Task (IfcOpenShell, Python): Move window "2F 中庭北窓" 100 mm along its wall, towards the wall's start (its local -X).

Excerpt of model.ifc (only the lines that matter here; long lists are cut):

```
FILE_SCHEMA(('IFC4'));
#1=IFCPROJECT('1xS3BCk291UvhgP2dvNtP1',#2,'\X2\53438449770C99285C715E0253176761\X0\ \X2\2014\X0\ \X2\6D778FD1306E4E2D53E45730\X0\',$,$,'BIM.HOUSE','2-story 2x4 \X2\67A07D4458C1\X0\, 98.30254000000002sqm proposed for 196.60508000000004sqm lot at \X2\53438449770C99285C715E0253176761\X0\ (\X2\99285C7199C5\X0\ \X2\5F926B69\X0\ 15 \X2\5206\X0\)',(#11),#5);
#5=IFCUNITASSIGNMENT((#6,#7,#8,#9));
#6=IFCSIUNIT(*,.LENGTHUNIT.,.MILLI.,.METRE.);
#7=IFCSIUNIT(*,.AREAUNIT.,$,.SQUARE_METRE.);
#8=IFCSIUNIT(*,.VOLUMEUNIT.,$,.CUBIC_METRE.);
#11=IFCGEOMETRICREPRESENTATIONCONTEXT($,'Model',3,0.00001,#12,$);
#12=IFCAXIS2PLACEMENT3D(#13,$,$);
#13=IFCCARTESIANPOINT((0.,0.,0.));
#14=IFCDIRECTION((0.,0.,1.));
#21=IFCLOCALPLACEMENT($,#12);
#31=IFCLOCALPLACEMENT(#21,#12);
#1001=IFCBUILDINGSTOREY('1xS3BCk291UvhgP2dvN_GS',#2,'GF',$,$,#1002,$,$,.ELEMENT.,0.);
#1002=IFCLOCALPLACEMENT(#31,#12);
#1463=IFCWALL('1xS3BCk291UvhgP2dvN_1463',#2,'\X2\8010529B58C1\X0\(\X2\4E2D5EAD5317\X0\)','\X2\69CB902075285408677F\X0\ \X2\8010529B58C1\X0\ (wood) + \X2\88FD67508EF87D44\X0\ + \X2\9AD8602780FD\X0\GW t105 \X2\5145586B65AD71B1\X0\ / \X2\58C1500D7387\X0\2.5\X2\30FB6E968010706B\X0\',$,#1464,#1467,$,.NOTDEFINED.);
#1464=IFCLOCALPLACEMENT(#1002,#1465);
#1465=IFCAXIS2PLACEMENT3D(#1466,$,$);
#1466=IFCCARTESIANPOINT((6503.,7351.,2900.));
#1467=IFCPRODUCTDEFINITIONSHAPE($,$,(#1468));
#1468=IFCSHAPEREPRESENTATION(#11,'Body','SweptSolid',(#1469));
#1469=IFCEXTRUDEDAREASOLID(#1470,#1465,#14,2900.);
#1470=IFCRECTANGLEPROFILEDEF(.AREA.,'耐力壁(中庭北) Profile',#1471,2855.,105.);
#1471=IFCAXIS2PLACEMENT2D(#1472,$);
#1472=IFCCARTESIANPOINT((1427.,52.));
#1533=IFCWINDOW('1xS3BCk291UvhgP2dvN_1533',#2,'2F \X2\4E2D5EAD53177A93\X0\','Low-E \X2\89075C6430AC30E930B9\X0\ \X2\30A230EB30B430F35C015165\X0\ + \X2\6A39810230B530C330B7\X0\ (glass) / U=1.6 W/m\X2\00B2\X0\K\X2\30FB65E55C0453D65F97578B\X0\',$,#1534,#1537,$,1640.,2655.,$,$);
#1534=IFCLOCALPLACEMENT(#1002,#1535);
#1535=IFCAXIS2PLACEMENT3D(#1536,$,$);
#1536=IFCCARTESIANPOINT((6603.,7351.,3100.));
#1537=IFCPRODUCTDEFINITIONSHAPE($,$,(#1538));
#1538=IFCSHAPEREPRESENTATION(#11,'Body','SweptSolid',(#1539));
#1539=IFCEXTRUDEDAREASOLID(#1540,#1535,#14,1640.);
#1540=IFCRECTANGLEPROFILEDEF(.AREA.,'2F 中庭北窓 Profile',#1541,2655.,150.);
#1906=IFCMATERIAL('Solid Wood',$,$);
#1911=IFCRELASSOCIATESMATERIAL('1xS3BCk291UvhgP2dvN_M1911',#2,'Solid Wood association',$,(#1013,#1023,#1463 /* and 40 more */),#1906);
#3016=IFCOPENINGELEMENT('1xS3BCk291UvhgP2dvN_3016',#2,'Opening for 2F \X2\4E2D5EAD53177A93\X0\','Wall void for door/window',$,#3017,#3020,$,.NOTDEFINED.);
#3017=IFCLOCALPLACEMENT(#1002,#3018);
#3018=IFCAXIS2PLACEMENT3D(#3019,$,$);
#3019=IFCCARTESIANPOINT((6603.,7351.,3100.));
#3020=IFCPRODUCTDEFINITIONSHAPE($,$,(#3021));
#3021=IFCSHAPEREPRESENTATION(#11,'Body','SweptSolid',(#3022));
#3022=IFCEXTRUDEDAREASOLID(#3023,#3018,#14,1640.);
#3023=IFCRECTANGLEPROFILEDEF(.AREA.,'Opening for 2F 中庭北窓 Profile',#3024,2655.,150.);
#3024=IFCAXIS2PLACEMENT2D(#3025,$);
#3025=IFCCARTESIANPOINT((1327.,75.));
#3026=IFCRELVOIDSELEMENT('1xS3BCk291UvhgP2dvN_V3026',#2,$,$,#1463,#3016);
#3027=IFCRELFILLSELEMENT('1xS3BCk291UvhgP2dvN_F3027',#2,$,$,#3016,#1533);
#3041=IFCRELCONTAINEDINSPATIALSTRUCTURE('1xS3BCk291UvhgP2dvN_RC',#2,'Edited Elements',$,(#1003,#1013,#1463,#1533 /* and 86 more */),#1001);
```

```python
import ifcopenshell
import ifcopenshell.api.geometry
import ifcopenshell.util.placement
import ifcopenshell.util.unit

model = ifcopenshell.open("model.ifc")
unit_scale = ifcopenshell.util.unit.calculate_unit_scale(model)

window = model.by_guid("1xS3BCk291UvhgP2dvN_1533")
opening = window.FillsVoids[0].RelatingOpeningElement
wall = opening.VoidsElements[0].RelatingBuildingElement

wall_matrix = ifcopenshell.util.placement.get_local_placement(wall.ObjectPlacement)
shift = wall_matrix[:3, 0] * -0.1 / unit_scale
before = ifcopenshell.util.placement.get_local_placement(window.ObjectPlacement)[:3, 3].copy()

# The window is not placed relative to its opening, so move both.
for product in (opening, window):
    matrix = ifcopenshell.util.placement.get_local_placement(product.ObjectPlacement)
    matrix[:3, 3] += shift
    ifcopenshell.api.geometry.edit_object_placement(model, product=product, matrix=matrix, is_si=False)

after = ifcopenshell.util.placement.get_local_placement(window.ObjectPlacement)[:3, 3]
print("window moved by", (after - before).round(3) + 0.0)

model.write("model-out.ifc")
```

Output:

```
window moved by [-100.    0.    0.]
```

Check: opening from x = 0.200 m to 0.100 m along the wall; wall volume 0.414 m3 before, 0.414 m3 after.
